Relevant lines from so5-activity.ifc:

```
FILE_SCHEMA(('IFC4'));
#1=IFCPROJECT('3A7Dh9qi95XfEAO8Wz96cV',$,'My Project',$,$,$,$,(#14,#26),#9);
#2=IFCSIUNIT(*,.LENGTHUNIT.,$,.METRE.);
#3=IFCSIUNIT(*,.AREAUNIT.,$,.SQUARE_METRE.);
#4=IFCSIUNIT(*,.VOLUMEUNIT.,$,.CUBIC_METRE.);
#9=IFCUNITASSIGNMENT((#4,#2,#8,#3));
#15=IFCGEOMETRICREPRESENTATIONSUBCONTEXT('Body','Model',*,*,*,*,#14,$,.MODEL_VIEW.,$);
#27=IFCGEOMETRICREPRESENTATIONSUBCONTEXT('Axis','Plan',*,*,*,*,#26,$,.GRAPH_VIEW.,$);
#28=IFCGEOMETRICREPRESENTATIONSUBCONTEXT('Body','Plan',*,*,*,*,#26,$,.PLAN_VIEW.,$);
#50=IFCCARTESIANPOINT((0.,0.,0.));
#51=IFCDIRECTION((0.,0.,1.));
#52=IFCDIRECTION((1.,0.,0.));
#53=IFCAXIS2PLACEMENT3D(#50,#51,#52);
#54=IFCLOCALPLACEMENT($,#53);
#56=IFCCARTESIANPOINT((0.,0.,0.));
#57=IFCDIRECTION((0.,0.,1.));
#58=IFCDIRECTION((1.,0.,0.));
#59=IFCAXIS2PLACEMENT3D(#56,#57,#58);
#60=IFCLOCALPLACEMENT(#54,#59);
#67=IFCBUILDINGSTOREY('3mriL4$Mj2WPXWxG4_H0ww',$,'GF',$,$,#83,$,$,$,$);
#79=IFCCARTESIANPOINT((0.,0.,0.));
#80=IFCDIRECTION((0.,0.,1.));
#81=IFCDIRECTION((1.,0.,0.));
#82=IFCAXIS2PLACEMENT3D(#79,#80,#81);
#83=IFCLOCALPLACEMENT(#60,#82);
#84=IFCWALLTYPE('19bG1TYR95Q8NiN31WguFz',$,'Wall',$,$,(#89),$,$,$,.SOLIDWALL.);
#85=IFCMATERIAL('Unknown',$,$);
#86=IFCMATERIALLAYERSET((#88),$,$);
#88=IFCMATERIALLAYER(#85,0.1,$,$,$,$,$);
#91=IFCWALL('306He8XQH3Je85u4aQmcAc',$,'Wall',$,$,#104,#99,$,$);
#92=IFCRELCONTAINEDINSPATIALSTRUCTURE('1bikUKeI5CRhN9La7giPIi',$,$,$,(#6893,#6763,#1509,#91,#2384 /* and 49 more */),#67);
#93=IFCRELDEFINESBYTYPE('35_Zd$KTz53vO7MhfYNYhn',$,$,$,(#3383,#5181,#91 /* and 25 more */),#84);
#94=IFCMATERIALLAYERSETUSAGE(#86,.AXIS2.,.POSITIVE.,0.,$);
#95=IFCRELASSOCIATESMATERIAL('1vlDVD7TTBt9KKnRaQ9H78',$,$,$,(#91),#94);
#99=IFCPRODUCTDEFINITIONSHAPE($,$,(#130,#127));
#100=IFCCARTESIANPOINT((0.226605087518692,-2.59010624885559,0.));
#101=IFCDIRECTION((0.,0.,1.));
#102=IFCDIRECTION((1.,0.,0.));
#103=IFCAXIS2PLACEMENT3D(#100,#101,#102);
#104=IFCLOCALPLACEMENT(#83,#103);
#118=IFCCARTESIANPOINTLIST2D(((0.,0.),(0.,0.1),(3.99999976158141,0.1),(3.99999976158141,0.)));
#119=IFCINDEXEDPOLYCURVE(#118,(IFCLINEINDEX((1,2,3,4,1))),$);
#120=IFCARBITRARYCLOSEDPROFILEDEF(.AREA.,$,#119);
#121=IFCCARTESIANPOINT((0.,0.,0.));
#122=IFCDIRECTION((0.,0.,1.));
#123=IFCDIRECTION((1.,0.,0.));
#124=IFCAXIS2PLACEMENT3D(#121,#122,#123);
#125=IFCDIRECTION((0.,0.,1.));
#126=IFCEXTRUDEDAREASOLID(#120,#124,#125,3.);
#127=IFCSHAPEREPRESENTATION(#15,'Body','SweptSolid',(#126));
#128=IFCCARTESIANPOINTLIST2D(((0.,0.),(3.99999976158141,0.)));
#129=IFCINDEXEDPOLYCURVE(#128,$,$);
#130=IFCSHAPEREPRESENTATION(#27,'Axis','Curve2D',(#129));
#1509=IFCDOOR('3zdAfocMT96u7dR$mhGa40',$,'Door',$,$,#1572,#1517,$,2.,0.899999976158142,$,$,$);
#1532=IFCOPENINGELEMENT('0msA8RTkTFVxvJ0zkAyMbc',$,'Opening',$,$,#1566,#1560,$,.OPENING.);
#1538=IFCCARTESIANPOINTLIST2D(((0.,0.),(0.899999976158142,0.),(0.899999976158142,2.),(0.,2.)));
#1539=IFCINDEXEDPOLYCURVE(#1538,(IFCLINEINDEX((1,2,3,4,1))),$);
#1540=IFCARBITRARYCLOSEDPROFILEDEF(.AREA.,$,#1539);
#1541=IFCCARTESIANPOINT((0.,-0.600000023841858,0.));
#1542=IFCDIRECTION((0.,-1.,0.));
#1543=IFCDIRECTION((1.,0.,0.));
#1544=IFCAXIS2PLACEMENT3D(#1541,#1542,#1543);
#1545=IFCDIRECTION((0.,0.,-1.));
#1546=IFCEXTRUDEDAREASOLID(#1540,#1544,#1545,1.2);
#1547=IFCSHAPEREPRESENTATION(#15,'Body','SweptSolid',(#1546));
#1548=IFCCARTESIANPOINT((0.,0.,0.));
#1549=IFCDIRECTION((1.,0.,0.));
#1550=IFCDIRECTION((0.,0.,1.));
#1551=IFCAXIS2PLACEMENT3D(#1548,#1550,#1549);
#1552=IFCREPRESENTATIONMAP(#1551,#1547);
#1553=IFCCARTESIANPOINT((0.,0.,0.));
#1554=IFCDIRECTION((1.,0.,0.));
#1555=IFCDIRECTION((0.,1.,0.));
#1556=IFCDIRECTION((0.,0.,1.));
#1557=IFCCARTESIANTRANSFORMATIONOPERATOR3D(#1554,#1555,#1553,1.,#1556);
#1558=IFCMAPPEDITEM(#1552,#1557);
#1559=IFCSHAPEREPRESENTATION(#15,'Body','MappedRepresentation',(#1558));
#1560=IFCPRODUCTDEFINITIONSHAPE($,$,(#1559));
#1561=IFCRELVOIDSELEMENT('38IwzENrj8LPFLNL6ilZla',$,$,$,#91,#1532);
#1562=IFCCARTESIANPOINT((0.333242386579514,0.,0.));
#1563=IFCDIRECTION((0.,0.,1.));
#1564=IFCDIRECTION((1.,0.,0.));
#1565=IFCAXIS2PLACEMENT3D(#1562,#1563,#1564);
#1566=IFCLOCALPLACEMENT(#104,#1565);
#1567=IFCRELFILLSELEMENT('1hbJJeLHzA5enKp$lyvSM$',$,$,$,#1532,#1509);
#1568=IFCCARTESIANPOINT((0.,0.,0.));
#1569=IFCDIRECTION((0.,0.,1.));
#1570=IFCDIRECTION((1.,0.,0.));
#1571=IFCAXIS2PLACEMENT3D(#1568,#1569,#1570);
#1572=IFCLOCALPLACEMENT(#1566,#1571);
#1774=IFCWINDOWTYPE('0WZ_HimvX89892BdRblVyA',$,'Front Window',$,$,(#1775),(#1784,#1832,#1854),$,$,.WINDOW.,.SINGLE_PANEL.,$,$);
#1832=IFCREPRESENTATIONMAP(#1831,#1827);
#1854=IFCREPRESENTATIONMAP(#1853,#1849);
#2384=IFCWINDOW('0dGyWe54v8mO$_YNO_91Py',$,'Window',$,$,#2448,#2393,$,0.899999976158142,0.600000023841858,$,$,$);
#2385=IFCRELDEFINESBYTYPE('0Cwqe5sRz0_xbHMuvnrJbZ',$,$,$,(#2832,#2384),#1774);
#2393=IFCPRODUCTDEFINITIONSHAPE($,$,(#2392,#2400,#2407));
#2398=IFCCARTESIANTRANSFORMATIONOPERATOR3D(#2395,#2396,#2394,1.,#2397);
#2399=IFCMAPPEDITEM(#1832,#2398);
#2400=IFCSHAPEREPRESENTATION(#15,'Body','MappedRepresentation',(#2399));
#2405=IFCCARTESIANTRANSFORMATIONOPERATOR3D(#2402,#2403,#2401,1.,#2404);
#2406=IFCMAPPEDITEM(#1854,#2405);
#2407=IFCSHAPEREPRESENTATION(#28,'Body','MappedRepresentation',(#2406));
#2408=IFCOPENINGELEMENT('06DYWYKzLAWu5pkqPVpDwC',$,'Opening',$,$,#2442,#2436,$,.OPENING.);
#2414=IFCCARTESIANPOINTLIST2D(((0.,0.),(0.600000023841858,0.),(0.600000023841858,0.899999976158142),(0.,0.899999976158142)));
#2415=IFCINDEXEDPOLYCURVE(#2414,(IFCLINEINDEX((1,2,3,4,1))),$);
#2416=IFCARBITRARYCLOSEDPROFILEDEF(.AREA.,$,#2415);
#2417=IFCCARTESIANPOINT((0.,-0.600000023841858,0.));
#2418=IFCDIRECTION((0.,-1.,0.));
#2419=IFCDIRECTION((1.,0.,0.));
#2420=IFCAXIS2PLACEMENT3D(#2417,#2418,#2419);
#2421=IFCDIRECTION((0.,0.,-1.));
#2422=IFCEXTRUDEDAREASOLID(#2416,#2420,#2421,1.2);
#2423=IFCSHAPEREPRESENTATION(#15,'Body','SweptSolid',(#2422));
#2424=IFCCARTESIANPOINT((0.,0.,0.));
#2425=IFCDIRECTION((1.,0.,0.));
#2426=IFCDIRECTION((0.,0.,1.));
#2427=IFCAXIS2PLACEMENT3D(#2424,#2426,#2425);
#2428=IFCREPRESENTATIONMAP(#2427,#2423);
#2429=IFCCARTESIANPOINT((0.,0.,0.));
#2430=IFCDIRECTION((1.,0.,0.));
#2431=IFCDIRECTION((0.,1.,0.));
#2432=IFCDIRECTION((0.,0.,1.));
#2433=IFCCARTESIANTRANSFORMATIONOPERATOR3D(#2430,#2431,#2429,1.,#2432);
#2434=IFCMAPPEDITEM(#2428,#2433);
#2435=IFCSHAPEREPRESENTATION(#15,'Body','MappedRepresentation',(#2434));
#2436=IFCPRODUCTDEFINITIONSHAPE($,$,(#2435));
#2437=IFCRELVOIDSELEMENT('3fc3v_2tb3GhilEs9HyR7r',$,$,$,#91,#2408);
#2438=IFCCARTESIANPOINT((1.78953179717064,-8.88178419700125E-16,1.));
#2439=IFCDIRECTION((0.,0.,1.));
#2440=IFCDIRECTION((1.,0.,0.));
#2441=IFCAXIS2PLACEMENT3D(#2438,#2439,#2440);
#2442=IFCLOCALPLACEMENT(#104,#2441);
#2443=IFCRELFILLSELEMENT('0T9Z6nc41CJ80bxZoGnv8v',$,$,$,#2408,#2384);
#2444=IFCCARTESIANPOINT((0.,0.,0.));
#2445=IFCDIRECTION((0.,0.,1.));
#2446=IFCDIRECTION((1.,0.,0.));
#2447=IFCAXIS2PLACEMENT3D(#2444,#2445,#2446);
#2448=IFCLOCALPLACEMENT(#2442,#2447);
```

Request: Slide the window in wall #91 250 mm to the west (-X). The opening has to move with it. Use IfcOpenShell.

```python
import ifcopenshell
import ifcopenshell.api.geometry
import ifcopenshell.util.placement
import ifcopenshell.util.unit

model = ifcopenshell.open("so5-activity.ifc")
unit_scale = ifcopenshell.util.unit.calculate_unit_scale(model)

window = model.by_id(2384)
opening = window.FillsVoids[0].RelatingOpeningElement
wall = opening.VoidsElements[0].RelatingBuildingElement

wall_matrix = ifcopenshell.util.placement.get_local_placement(wall.ObjectPlacement)
shift = wall_matrix[:3, 0] * -0.25 / unit_scale
before = ifcopenshell.util.placement.get_local_placement(window.ObjectPlacement)[:3, 3].copy()

# The window is placed relative to its opening, so it follows when the opening moves.
matrix = ifcopenshell.util.placement.get_local_placement(opening.ObjectPlacement)
matrix[:3, 3] += shift
ifcopenshell.api.geometry.edit_object_placement(
    model, product=opening, matrix=matrix, is_si=False, should_transform_children=True
)

after = ifcopenshell.util.placement.get_local_placement(window.ObjectPlacement)[:3, 3]
print("window moved by", (after - before).round(3) + 0.0)

model.write("so5-activity_rev.ifc")
```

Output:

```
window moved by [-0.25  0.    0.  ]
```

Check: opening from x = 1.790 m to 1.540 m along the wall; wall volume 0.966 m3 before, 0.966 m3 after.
